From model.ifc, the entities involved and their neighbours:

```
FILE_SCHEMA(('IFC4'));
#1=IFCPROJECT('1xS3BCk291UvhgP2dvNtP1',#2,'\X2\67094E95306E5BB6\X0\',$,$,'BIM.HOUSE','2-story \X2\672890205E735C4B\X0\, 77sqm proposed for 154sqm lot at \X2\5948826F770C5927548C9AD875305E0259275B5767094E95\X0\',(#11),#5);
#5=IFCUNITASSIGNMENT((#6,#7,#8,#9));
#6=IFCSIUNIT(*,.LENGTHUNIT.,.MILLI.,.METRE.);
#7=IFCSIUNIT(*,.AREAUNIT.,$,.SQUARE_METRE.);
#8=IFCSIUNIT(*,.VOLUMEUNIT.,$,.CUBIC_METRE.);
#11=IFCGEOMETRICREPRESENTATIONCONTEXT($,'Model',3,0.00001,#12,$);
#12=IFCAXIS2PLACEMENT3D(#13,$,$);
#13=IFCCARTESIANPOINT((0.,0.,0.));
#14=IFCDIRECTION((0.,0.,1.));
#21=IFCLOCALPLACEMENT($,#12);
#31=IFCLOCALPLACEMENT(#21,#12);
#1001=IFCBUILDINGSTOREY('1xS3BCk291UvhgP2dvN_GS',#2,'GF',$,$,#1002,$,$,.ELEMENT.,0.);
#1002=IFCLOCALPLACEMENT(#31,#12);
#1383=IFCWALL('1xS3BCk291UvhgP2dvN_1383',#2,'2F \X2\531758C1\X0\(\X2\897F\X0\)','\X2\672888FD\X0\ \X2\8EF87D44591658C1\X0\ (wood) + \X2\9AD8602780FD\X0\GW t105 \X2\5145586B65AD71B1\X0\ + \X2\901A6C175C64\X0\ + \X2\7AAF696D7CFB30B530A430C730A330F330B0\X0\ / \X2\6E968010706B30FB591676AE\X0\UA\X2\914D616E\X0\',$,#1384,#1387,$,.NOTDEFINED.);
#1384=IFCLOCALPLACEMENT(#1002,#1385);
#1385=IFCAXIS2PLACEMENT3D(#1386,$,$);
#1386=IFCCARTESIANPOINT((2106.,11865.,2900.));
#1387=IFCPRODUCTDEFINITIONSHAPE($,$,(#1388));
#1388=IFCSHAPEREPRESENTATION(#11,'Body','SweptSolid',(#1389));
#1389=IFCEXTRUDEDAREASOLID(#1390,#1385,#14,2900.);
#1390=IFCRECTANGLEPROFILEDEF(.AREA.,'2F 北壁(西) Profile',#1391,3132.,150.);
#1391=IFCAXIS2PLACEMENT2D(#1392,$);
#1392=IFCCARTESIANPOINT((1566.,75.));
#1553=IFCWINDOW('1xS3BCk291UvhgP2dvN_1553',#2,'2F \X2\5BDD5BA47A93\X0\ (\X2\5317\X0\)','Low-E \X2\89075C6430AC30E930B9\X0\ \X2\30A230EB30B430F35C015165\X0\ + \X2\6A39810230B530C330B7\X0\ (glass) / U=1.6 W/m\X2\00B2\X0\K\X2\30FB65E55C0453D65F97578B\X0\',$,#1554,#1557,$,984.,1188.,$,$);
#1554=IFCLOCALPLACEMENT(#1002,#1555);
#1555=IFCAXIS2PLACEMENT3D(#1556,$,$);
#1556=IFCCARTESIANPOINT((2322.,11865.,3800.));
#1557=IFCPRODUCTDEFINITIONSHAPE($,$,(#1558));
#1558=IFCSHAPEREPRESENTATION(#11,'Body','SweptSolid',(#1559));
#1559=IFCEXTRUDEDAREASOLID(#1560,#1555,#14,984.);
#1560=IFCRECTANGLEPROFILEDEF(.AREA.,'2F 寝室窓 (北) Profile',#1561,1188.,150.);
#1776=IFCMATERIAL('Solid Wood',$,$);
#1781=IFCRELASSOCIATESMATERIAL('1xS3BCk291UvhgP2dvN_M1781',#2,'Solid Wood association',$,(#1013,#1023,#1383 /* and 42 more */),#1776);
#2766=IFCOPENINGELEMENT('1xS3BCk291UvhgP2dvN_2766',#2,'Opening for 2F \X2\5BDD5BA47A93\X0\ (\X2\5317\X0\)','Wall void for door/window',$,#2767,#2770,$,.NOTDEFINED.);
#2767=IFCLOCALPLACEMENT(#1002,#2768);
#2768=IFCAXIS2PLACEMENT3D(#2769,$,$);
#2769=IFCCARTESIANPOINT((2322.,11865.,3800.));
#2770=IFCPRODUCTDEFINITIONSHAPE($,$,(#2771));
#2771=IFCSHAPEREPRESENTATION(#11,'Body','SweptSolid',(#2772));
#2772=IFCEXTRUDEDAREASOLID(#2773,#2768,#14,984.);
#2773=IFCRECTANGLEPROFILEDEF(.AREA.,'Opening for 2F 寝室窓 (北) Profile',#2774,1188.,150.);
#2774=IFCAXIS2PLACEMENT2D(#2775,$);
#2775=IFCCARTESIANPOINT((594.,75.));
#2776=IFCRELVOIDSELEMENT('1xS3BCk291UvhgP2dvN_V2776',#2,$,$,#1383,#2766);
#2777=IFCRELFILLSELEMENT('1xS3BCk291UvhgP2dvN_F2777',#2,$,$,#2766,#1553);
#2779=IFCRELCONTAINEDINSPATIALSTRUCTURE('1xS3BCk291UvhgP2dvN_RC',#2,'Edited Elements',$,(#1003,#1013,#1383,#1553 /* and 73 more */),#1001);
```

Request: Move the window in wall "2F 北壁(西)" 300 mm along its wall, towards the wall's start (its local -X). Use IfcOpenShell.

```python
import ifcopenshell
import ifcopenshell.api.geometry
import ifcopenshell.util.placement
import ifcopenshell.util.unit

model = ifcopenshell.open("model.ifc")
unit_scale = ifcopenshell.util.unit.calculate_unit_scale(model)

window = model.by_guid("1xS3BCk291UvhgP2dvN_1553")
opening = window.FillsVoids[0].RelatingOpeningElement
wall = opening.VoidsElements[0].RelatingBuildingElement

wall_matrix = ifcopenshell.util.placement.get_local_placement(wall.ObjectPlacement)
shift = wall_matrix[:3, 0] * -0.3 / unit_scale
before = ifcopenshell.util.placement.get_local_placement(window.ObjectPlacement)[:3, 3].copy()

# The window is not placed relative to its opening, so move both.
for product in (opening, window):
    matrix = ifcopenshell.util.placement.get_local_placement(product.ObjectPlacement)
    matrix[:3, 3] += shift
    ifcopenshell.api.geometry.edit_object_placement(model, product=product, matrix=matrix, is_si=False)

after = ifcopenshell.util.placement.get_local_placement(window.ObjectPlacement)[:3, 3]
print("window moved by", (after - before).round(3) + 0.0)

model.write("model-out.ifc")
```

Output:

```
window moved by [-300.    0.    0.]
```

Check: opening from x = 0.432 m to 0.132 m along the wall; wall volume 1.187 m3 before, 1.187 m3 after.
